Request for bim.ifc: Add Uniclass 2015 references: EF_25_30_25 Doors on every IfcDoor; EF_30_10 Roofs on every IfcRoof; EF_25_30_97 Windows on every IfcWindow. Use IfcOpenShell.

First a look at what the model holds.

```python
import ifcopenshell

model = ifcopenshell.open("bim.ifc")
print(model.schema)
print("classifications:", [c.Name for c in model.by_type("IfcClassification")])
for ifc_class in ("IfcDoor", "IfcRoof", "IfcStair", "IfcWall", "IfcWindow"):
    print(ifc_class, len(model.by_type(ifc_class)))
```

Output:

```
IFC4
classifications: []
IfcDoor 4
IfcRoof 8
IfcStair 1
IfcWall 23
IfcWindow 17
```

```python
import ifcopenshell
import ifcopenshell.api.classification

model = ifcopenshell.open("bim.ifc")

system = ifcopenshell.api.classification.add_classification(model, classification="Uniclass 2015")

codes = {
    "IfcDoor": ("EF_25_30_25", "Doors"),
    "IfcRoof": ("EF_30_10", "Roofs"),
    "IfcWindow": ("EF_25_30_97", "Windows"),
}
for ifc_class, (code, name) in codes.items():
    products = model.by_type(ifc_class)
    ifcopenshell.api.classification.add_reference(
        model, products=products, classification=system, identification=code, name=name
    )
    print(code, len(products))

model.write("bim_rev.ifc")
```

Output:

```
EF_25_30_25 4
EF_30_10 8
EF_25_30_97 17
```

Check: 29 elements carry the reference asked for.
